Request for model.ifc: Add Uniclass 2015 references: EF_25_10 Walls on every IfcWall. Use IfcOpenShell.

First a look at what the model holds.

```python
import ifcopenshell

model = ifcopenshell.open("model.ifc")
print(model.schema)
print("classifications:", [c.Name for c in model.by_type("IfcClassification")])
for ifc_class in ("IfcDoor", "IfcRoof", "IfcStair", "IfcWall", "IfcWindow"):
    print(ifc_class, len(model.by_type(ifc_class)))
```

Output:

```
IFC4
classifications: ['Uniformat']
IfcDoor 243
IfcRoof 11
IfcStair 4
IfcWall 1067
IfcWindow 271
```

```python
import ifcopenshell
import ifcopenshell.api.classification

model = ifcopenshell.open("model.ifc")

system = ifcopenshell.api.classification.add_classification(model, classification="Uniclass 2015")

codes = {
    "IfcWall": ("EF_25_10", "Walls"),
}
for ifc_class, (code, name) in codes.items():
    products = model.by_type(ifc_class)
    ifcopenshell.api.classification.add_reference(
        model, products=products, classification=system, identification=code, name=name
    )
    print(code, len(products))

model.write("model_v2.ifc")
```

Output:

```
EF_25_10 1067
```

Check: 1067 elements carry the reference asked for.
